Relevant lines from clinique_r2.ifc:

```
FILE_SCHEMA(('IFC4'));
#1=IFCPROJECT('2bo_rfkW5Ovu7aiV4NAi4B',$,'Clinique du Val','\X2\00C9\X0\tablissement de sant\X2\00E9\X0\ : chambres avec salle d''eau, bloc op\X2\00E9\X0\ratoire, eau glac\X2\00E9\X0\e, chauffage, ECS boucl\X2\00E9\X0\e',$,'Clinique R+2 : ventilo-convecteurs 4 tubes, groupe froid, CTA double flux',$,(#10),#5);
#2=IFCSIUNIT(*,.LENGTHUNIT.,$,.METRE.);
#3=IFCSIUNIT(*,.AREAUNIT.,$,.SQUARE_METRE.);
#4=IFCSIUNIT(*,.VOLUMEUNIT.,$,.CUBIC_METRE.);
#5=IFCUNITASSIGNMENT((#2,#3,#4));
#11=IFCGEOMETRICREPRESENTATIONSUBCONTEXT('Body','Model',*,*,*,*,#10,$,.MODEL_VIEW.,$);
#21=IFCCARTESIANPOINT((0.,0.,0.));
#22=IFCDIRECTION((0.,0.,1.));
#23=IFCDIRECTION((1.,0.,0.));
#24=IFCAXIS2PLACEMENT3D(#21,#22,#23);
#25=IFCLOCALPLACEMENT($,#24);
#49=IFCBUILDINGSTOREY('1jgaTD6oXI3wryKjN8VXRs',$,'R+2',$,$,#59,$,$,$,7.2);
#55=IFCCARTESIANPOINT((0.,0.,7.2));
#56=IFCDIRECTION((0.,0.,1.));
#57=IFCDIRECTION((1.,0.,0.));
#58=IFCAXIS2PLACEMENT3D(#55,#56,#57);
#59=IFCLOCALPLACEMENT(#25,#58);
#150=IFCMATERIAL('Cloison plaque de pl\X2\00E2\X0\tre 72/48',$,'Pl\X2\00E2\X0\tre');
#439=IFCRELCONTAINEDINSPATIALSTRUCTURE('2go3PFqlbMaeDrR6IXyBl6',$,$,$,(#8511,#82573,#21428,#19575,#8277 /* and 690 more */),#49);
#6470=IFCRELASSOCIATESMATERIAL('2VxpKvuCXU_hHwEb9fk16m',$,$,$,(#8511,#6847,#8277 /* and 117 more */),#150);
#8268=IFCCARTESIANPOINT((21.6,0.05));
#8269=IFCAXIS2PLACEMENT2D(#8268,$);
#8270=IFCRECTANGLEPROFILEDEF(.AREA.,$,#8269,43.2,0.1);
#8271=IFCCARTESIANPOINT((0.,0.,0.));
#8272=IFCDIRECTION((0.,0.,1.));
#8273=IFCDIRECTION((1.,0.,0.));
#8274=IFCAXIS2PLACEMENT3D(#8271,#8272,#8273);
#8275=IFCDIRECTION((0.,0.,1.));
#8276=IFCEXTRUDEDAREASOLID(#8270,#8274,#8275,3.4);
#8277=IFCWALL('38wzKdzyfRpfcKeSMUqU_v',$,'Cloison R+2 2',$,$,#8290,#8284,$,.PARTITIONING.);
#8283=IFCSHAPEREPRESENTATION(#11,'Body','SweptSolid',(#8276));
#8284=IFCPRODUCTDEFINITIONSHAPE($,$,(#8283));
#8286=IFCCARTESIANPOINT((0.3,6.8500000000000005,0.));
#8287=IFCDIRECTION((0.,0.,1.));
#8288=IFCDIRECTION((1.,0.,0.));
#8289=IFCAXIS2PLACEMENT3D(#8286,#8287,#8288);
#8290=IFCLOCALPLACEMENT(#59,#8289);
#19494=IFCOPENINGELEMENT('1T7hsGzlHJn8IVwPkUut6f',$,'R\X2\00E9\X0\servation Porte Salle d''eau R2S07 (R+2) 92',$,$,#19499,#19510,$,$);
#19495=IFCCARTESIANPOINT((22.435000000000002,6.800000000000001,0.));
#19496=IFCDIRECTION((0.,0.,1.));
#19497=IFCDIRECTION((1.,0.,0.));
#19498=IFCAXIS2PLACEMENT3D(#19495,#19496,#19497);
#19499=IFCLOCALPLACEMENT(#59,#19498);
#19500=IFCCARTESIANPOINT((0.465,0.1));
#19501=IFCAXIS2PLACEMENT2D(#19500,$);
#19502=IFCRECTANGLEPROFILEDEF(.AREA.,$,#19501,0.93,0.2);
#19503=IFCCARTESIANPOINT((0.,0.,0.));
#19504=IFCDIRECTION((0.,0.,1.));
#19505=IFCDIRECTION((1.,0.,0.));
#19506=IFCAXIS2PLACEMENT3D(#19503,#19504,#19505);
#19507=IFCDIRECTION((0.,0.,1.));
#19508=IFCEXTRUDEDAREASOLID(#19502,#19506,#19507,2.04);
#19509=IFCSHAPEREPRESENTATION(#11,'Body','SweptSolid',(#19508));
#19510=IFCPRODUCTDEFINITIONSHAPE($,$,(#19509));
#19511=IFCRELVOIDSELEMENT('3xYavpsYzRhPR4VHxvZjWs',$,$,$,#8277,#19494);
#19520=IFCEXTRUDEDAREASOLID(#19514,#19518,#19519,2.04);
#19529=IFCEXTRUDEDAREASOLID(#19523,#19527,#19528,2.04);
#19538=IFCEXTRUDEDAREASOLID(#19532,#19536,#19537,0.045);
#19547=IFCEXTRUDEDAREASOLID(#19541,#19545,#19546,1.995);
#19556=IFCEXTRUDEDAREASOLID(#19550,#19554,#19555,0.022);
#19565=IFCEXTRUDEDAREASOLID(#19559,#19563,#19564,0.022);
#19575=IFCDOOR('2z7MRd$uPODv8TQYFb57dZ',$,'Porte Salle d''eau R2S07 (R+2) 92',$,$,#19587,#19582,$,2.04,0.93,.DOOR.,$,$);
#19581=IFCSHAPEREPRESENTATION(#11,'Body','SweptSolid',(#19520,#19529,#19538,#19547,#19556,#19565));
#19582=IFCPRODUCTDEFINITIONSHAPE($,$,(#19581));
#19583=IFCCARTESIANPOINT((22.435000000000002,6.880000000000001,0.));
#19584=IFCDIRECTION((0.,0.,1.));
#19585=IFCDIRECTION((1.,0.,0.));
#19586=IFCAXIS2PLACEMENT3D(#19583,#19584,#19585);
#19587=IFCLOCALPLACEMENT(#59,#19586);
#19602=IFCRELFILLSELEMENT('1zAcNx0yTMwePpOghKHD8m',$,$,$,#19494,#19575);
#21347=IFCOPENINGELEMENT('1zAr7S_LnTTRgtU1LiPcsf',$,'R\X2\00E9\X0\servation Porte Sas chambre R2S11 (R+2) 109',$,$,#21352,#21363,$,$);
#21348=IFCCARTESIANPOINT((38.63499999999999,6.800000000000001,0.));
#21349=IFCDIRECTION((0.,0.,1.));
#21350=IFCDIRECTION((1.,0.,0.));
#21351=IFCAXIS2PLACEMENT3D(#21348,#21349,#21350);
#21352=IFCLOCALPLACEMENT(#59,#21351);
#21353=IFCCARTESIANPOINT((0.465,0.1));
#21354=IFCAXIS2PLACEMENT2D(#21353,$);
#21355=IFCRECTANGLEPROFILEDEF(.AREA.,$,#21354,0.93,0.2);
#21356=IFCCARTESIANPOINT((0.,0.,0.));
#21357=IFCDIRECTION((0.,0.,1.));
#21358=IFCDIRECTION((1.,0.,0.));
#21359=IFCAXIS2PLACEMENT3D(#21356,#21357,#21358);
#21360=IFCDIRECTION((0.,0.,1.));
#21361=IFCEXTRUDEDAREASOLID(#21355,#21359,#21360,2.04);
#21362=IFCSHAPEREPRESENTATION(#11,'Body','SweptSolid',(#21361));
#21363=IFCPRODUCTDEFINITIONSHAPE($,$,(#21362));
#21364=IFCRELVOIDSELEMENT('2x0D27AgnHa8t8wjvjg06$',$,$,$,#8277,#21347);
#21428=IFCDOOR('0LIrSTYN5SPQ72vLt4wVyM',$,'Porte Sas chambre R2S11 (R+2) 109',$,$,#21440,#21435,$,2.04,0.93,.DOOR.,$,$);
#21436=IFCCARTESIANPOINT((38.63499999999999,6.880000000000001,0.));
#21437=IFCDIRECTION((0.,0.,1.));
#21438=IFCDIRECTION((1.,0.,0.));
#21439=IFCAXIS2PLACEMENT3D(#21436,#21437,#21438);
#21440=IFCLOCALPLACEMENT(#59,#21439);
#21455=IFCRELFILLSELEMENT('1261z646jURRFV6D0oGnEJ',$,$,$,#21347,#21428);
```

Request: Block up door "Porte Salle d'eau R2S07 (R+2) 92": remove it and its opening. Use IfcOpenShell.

```python
import ifcopenshell
import ifcopenshell.api.feature
import ifcopenshell.api.root
import ifcopenshell.geom
import ifcopenshell.util.shape

model = ifcopenshell.open("clinique_r2.ifc")
settings = ifcopenshell.geom.settings()


def volume(element):
    """Net volume in cubic metres, openings subtracted."""
    shape = ifcopenshell.geom.create_shape(settings, element)
    return ifcopenshell.util.shape.get_volume(shape.geometry)


door = model.by_id(19575)
opening = door.FillsVoids[0].RelatingOpeningElement
wall = opening.VoidsElements[0].RelatingBuildingElement
before = volume(wall)

ifcopenshell.api.root.remove_product(model, product=door)
ifcopenshell.api.feature.remove_feature(model, feature=opening)

after = volume(wall)

print(f"wall volume {before:.3f} -> {after:.3f} m3")

model.write("clinique_r2_rev.ifc")
```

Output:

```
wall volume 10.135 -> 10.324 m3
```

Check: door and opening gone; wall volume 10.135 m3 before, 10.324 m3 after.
